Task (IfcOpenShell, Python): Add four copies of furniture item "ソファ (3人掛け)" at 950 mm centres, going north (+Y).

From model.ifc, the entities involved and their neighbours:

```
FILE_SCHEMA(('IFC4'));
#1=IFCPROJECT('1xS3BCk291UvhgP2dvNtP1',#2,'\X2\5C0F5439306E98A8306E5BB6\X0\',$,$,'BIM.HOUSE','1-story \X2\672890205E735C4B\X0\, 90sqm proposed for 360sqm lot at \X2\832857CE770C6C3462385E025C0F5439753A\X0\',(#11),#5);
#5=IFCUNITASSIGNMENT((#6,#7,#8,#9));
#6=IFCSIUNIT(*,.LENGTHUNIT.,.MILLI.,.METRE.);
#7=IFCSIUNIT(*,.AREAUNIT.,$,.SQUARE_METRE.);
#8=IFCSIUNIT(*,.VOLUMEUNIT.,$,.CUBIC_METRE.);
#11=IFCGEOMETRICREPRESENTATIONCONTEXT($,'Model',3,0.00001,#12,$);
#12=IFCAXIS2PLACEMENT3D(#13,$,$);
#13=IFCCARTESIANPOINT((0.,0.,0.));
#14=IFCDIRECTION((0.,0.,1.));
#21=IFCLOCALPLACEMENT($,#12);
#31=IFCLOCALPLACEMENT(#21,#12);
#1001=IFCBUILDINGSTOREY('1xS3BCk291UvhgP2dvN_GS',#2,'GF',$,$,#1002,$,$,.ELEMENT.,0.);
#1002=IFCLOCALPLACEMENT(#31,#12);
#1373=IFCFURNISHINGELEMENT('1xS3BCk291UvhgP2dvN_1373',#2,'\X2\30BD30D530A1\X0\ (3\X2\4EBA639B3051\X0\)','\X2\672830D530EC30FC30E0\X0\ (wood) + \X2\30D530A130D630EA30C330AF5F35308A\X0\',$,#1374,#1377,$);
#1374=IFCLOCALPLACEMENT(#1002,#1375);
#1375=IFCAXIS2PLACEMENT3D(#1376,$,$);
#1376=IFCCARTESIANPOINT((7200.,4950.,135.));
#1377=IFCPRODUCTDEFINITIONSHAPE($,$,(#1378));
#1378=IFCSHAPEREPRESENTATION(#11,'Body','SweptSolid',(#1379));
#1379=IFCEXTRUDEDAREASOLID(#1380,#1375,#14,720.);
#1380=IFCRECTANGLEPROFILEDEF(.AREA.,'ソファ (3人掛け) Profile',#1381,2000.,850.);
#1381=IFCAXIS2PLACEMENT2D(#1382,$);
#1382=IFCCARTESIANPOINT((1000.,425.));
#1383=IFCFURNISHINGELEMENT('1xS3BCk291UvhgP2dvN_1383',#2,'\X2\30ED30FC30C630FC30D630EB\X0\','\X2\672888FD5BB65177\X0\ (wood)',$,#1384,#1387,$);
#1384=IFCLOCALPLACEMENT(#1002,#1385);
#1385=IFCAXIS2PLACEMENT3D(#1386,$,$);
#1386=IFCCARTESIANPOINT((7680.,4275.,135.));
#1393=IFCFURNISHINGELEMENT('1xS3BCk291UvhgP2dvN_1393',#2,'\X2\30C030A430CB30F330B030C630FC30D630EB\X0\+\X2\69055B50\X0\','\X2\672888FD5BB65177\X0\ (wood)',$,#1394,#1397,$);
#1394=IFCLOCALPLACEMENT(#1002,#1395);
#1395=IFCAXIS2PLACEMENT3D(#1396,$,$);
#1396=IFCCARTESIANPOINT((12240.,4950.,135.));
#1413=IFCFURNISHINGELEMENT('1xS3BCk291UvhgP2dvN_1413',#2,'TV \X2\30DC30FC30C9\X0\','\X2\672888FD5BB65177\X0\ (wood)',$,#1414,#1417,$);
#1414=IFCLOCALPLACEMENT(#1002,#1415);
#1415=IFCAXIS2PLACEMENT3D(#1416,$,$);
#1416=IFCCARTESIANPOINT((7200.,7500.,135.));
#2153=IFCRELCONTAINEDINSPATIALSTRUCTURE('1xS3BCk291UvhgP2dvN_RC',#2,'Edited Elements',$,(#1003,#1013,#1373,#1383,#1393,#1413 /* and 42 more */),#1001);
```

```python
import numpy as np
import ifcopenshell
import ifcopenshell.api.geometry
import ifcopenshell.api.root
import ifcopenshell.util.element
import ifcopenshell.util.placement

model = ifcopenshell.open("model.ifc")


def reuse_history(source, copy):
    """copy_class also copies each property set's owner history, people and application; keep the originals."""
    for rel in copy.IsDefinedBy:
        if rel.is_a("IfcRelDefinesByProperties") and (history := rel.RelatingPropertyDefinition.OwnerHistory):
            rel.RelatingPropertyDefinition.OwnerHistory = source.OwnerHistory
            ifcopenshell.util.element.remove_deep2(model, history)


source = model.by_guid("1xS3BCk291UvhgP2dvN_1373")
base = ifcopenshell.util.placement.get_local_placement(source.ObjectPlacement)
step = np.array([0.0, 1.0, 0.0]) * 950.0

for i in range(1, 5):
    copy = ifcopenshell.api.root.copy_class(model, product=source)
    copy.Representation = ifcopenshell.util.element.copy_deep(
        model, source.Representation, exclude=["IfcGeometricRepresentationContext", "IfcRepresentationMap"]
    )
    reuse_history(source, copy)
    matrix = base.copy()
    matrix[:3, 3] += i * step
    print("added at", matrix[:3, 3].round(3) + 0.0)
    ifcopenshell.api.geometry.edit_object_placement(model, product=copy, matrix=matrix, is_si=False)

model.write("model_edited.ifc")
```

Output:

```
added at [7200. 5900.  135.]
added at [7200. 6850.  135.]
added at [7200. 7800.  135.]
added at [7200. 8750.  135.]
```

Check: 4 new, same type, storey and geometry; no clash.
